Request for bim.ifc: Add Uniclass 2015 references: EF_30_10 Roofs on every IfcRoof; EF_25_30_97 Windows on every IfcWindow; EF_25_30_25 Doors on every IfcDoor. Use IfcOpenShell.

First a look at what the model holds.

```python
import ifcopenshell

model = ifcopenshell.open("bim.ifc")
print(model.schema)
print("classifications:", [c.Name for c in model.by_type("IfcClassification")])
for ifc_class in ("IfcDoor", "IfcRoof", "IfcStair", "IfcWall", "IfcWindow"):
    print(ifc_class, len(model.by_type(ifc_class)))
```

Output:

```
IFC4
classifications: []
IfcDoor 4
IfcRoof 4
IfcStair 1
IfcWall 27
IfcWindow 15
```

```python
import ifcopenshell
import ifcopenshell.api.classification

model = ifcopenshell.open("bim.ifc")

system = ifcopenshell.api.classification.add_classification(model, classification="Uniclass 2015")

codes = {
    "IfcRoof": ("EF_30_10", "Roofs"),
    "IfcWindow": ("EF_25_30_97", "Windows"),
    "IfcDoor": ("EF_25_30_25", "Doors"),
}
for ifc_class, (code, name) in codes.items():
    products = model.by_type(ifc_class)
    ifcopenshell.api.classification.add_reference(
        model, products=products, classification=system, identification=code, name=name
    )
    print(code, len(products))

model.write("bim_updated.ifc")
```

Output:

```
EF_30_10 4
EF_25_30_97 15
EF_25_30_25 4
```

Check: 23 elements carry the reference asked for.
